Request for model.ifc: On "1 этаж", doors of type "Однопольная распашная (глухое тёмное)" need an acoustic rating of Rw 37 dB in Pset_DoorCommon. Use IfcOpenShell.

First a look at what the model holds.

```python
import ifcopenshell
import ifcopenshell.util.element

model = ifcopenshell.open("model.ifc")
print(model.schema)
storey = next(s for s in model.by_type("IfcBuildingStorey") if s.Name == "1 этаж")
doors = [e for e in ifcopenshell.util.element.get_decomposition(storey) if e.is_a("IfcDoor")]
seen = {}
for e in doors:
    element_type = ifcopenshell.util.element.get_type(e)
    key = (element_type.Name if element_type != e and element_type else None, ifcopenshell.util.element.get_pset(e, "Pset_DoorCommon", "AcousticRating"))
    seen[key] = seen.get(key, 0) + 1
for (name, value), count in sorted(seen.items(), key=str):
    print(count, "x", name, "|", value)
```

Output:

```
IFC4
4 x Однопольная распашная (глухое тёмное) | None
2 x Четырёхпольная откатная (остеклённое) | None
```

```python
import ifcopenshell
import ifcopenshell.api.pset
import ifcopenshell.util.element

model = ifcopenshell.open("model.ifc")

storey = next(s for s in model.by_type("IfcBuildingStorey") if s.Name == "1 этаж")
doors = [e for e in ifcopenshell.util.element.get_decomposition(storey) if e.is_a("IfcDoor")]

count = 0
for e in doors:
    element_type = ifcopenshell.util.element.get_type(e)
    if element_type in (None, e) or element_type.Name != "Однопольная распашная (глухое тёмное)":
        continue
    # add_pset returns the element's existing set when there is one.
    pset = ifcopenshell.api.pset.add_pset(model, product=e, name="Pset_DoorCommon")
    ifcopenshell.api.pset.edit_pset(model, pset=pset, properties={"AcousticRating": "Rw 37 dB"})
    count += 1

print(count, "doors updated")

model.write("model-out.ifc")
```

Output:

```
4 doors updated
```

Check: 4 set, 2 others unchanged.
